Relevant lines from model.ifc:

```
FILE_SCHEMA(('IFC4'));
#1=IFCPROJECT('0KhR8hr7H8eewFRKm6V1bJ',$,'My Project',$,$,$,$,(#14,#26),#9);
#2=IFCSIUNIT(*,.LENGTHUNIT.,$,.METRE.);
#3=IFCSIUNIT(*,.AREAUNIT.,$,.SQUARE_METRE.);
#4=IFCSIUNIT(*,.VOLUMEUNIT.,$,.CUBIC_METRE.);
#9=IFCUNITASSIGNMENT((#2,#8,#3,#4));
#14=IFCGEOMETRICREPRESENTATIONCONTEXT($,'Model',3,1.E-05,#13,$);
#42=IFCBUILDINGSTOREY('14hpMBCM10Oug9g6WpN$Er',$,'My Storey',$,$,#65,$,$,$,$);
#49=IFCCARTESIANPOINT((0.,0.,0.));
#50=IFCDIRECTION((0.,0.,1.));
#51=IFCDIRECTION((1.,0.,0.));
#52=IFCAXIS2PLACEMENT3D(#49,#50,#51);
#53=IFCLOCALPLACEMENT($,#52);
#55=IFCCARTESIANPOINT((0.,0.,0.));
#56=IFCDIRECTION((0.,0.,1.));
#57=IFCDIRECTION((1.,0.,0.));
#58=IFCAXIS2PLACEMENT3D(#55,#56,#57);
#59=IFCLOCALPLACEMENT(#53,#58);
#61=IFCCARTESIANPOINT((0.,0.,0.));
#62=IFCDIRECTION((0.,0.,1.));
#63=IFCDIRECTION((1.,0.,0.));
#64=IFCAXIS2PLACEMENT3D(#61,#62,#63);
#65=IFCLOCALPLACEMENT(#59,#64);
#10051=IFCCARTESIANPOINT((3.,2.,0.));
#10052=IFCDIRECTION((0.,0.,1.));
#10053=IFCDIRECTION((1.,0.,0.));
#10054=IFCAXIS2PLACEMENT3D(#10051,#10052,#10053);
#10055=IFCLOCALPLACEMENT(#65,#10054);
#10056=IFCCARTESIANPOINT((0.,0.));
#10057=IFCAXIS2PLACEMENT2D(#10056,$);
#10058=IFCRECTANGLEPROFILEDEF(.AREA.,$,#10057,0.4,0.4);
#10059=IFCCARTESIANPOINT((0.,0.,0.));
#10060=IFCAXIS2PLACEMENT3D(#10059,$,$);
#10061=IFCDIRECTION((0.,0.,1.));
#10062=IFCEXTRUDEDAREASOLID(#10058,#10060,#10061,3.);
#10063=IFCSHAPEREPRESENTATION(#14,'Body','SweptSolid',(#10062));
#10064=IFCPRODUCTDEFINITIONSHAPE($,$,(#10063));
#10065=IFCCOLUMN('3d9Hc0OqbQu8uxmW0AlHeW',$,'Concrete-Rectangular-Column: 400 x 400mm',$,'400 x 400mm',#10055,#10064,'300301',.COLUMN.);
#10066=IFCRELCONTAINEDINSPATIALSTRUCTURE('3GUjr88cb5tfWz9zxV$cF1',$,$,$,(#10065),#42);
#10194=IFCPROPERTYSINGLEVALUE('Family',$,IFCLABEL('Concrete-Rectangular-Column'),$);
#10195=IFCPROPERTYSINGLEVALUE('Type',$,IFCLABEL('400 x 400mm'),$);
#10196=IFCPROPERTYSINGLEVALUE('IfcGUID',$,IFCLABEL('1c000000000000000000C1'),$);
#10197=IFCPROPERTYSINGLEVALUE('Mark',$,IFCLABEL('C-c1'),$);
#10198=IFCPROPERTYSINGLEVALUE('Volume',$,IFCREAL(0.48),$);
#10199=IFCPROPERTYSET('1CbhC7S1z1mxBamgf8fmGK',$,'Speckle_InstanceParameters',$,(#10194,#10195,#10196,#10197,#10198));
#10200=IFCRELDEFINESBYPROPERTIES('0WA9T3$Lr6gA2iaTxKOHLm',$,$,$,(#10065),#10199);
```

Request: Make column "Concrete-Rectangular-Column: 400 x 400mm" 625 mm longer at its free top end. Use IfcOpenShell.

```python
import ifcopenshell
import ifcopenshell.api.pset
import ifcopenshell.util.element
import ifcopenshell.util.unit

model = ifcopenshell.open("model.ifc")
unit_scale = ifcopenshell.util.unit.calculate_unit_scale(model)

member = model.by_guid("3d9Hc0OqbQu8uxmW0AlHeW")
change = 0.625 / unit_scale

# The extrusion runs towards the end named, so only its depth changes.
body = next(r for r in member.Representation.Representations if r.RepresentationIdentifier == "Body")
solid = body.Items[0]
old_length = solid.Depth
solid.Depth += change

# Update the stored length and volume.
pset = model.by_id(ifcopenshell.util.element.get_pset(member, "Speckle_InstanceParameters", should_inherit=False)["id"])
ifcopenshell.api.pset.edit_pset(model, pset=pset, properties={
    "Volume": model.create_entity("IfcReal", ifcopenshell.util.element.get_pset(member, "Speckle_InstanceParameters", "Volume") * solid.Depth / old_length),
})

print(f"length {old_length:g} -> {solid.Depth:g}")

model.write("model_rev.ifc")
```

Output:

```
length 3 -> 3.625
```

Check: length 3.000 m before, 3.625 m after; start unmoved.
